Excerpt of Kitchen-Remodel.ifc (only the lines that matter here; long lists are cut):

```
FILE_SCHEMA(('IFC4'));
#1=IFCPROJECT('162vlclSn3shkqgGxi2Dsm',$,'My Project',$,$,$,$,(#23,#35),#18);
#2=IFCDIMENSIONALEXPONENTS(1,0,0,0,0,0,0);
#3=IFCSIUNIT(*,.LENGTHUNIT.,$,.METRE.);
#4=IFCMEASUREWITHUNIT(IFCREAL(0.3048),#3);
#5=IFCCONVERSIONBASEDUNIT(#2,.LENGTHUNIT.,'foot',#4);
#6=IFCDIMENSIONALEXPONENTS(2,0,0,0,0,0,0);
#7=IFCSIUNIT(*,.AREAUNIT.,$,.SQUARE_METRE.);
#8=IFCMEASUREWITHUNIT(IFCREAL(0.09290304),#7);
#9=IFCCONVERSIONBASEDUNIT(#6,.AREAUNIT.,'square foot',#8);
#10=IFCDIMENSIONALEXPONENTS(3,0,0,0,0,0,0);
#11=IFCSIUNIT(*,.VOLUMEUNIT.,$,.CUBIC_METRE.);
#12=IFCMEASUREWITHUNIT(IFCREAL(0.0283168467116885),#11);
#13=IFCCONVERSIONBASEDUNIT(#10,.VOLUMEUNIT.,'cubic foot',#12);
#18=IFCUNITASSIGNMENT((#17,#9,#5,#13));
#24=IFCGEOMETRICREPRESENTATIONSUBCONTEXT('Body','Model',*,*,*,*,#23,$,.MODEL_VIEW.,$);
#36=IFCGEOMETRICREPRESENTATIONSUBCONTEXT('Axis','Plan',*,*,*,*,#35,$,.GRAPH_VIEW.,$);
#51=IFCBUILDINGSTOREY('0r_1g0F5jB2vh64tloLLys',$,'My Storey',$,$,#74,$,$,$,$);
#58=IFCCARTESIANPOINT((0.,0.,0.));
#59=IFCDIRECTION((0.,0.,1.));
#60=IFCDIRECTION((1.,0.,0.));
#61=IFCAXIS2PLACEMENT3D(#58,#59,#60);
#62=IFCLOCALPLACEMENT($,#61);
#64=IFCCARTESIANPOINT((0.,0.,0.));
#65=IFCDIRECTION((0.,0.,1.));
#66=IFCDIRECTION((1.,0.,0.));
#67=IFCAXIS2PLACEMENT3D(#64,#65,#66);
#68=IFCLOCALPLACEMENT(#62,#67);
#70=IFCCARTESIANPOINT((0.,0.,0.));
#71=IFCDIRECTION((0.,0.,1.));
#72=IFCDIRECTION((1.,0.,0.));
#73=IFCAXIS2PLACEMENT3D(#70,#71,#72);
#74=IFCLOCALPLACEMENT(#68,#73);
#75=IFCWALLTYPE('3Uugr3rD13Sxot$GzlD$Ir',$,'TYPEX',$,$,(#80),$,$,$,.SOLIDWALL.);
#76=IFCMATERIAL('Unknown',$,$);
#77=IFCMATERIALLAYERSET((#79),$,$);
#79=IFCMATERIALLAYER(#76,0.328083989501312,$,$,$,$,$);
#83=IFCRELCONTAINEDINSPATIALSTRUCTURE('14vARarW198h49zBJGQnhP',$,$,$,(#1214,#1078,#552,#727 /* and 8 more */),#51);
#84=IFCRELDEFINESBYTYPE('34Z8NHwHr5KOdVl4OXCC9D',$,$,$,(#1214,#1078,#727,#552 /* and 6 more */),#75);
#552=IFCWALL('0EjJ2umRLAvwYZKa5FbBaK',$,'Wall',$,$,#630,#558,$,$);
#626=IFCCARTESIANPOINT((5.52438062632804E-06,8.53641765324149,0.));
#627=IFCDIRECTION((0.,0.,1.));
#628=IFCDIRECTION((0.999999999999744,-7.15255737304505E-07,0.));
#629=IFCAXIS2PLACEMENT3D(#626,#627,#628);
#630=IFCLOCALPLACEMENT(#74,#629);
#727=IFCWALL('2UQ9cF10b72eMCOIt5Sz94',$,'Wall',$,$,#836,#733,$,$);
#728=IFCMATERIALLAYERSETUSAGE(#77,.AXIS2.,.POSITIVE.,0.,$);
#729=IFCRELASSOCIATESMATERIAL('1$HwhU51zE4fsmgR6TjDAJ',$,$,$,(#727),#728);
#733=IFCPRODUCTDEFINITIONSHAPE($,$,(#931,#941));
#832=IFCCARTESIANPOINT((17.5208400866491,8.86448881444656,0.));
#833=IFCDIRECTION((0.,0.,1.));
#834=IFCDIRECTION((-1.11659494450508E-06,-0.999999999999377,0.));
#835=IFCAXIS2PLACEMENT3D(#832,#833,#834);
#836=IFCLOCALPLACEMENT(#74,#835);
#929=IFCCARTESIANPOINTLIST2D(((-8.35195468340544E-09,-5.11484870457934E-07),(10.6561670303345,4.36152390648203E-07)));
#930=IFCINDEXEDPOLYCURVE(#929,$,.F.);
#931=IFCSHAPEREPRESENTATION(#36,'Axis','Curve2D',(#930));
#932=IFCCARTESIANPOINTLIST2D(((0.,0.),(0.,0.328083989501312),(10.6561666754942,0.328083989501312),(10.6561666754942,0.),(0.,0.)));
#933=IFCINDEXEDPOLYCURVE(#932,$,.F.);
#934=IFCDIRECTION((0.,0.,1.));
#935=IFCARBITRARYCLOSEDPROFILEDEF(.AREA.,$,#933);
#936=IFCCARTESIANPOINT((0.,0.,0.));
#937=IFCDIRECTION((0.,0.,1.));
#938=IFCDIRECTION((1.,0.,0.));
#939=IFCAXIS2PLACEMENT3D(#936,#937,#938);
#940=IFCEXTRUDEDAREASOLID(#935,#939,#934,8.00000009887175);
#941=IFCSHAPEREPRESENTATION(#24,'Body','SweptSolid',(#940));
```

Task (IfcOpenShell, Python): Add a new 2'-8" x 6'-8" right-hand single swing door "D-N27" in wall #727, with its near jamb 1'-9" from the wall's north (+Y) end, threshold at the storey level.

```python
import numpy as np
import ifcopenshell
import ifcopenshell.api.feature
import ifcopenshell.api.geometry
import ifcopenshell.api.root
import ifcopenshell.api.spatial
import ifcopenshell.geom
import ifcopenshell.util.element
import ifcopenshell.util.placement
import ifcopenshell.util.representation
import ifcopenshell.util.shape
import ifcopenshell.util.unit

model = ifcopenshell.open("Kitchen-Remodel.ifc")
unit_scale = ifcopenshell.util.unit.calculate_unit_scale(model)
settings = ifcopenshell.geom.settings()


def volume(element):
    """Net volume in cubic metres, openings subtracted."""
    shape = ifcopenshell.geom.create_shape(settings, element)
    return ifcopenshell.util.shape.get_volume(shape.geometry)


wall = model.by_guid("2UQ9cF10b72eMCOIt5Sz94")
storey = ifcopenshell.util.element.get_container(wall, ifc_class="IfcBuildingStorey")
context = ifcopenshell.util.representation.get_context(model, "Model", "Body", "MODEL_VIEW")
before = volume(wall)

width, height, from_end, sill = 0.8128, 2.032, 0.5334, 0.0  # metres

# The wall runs along its own X axis, and the end named is its -X end.
wall_shape = ifcopenshell.geom.create_shape(settings, wall)
x, y, z = ifcopenshell.util.shape.get_vertices(wall_shape.geometry).T
start = x.min() + from_end
face, thickness = float(y.min()), float(y.max() - y.min())
wall_matrix = ifcopenshell.util.placement.get_local_placement(wall.ObjectPlacement)
level = ifcopenshell.util.placement.get_local_placement(storey.ObjectPlacement)[2, 3]


def in_wall(x, y):
    """Placement at x, y metres in the wall's axes, at sill height."""
    matrix = wall_matrix.copy()
    matrix[:, 3] = wall_matrix @ np.array([x / unit_scale, y / unit_scale, 0.0, 1.0])
    matrix[2, 3] = level + sill / unit_scale
    return matrix


# Opening: a box that overshoots both wall faces by 50 mm.
opening = ifcopenshell.api.root.create_entity(model, ifc_class="IfcOpeningElement", predefined_type="OPENING")
box = ifcopenshell.api.geometry.add_wall_representation(
    model, context=context, length=width, height=height, thickness=thickness + 0.1
)
ifcopenshell.api.geometry.assign_representation(model, product=opening, representation=box)
ifcopenshell.api.geometry.edit_object_placement(model, product=opening, matrix=in_wall(start, face - 0.05), is_si=False)
ifcopenshell.api.feature.add_feature(model, feature=opening, element=wall)

door = ifcopenshell.api.root.create_entity(model, ifc_class="IfcDoor", name="D-N27", predefined_type="DOOR")
door.OverallWidth, door.OverallHeight = width / unit_scale, height / unit_scale
door.OperationType = "SINGLE_SWING_RIGHT"
body = ifcopenshell.api.geometry.add_door_representation(
    model,
    context=context,
    overall_width=door.OverallWidth,
    overall_height=door.OverallHeight,
    operation_type="SINGLE_SWING_RIGHT",
    lining_properties={"LiningDepth": thickness / unit_scale, "ThresholdDepth": thickness / unit_scale},
)
ifcopenshell.api.geometry.assign_representation(model, product=door, representation=body)
ifcopenshell.api.spatial.assign_container(model, products=[door], relating_structure=storey)
ifcopenshell.api.feature.add_filling(model, opening=opening, element=door)

# The lining spans the wall, so the door starts at the wall face.
ifcopenshell.api.geometry.edit_object_placement(model, product=door, matrix=in_wall(start, face), is_si=False)

after = volume(wall)

print(f"wall volume {before:.3f} -> {after:.3f} m3")

model.write("Kitchen-Remodel-out.ifc")
```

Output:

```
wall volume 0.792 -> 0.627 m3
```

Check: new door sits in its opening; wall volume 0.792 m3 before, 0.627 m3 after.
